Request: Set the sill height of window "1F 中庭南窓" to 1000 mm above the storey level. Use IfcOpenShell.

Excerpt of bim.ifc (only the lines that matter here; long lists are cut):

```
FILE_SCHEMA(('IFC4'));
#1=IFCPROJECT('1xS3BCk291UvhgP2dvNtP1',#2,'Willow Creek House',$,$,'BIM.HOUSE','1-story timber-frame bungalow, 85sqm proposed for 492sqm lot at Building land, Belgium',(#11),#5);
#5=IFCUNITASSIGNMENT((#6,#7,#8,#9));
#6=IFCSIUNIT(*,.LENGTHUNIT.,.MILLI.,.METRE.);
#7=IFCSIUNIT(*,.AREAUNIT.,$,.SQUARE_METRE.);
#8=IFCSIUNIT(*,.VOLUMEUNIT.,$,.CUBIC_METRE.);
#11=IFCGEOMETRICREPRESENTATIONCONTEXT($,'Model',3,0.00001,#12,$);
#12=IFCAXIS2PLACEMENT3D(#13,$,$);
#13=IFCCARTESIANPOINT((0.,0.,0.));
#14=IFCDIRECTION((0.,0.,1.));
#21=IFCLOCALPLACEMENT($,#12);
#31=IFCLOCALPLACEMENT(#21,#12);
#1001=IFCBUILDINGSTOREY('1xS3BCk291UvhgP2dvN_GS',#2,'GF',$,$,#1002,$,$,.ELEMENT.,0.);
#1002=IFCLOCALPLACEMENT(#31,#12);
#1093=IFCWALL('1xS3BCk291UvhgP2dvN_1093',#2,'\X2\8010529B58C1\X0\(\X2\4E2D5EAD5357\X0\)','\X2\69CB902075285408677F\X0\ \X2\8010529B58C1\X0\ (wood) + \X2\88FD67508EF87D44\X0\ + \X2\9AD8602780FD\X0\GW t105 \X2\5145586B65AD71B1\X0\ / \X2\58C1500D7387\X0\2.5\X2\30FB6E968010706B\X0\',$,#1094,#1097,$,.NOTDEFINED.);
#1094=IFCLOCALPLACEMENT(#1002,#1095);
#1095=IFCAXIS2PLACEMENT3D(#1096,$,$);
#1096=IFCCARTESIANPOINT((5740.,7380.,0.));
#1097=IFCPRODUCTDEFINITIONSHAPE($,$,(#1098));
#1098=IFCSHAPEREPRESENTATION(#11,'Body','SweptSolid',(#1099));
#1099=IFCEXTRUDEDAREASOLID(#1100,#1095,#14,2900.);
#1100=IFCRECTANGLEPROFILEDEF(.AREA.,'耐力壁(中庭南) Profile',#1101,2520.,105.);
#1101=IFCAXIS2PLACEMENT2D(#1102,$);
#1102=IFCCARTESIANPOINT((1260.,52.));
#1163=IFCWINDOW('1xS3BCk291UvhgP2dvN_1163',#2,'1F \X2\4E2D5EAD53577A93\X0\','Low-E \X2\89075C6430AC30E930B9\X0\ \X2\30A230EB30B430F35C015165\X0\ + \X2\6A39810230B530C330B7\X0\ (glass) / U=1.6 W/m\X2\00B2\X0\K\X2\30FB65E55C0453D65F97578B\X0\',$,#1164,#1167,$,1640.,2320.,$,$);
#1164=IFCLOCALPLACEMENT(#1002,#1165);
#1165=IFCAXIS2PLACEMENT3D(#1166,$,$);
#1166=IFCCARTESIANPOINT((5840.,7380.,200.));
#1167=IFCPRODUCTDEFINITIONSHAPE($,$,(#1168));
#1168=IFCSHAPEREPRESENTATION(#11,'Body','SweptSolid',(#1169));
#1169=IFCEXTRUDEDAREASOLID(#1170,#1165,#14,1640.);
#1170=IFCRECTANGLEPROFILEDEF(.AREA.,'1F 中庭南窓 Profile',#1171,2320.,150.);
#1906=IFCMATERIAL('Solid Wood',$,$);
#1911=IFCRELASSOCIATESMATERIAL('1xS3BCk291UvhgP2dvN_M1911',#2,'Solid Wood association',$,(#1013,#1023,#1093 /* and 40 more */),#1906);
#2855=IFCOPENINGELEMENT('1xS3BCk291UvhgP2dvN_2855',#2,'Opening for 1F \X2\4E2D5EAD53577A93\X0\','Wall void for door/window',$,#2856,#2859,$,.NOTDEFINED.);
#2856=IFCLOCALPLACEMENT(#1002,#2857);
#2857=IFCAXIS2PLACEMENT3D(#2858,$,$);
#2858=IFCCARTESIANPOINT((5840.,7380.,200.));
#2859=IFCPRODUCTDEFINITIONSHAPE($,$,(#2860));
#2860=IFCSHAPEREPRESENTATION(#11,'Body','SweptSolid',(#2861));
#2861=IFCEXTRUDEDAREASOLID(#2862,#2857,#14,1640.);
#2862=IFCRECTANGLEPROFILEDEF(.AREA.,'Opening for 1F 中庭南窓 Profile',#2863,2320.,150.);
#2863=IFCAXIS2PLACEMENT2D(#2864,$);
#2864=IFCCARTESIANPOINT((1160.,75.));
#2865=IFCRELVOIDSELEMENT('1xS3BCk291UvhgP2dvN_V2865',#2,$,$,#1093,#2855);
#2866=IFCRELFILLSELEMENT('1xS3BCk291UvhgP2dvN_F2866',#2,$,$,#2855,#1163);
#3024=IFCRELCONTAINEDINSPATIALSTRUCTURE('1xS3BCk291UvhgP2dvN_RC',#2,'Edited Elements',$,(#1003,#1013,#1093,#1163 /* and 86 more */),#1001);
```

```python
import numpy as np
import ifcopenshell
import ifcopenshell.api.geometry
import ifcopenshell.geom
import ifcopenshell.util.element
import ifcopenshell.util.placement
import ifcopenshell.util.shape
import ifcopenshell.util.unit

model = ifcopenshell.open("bim.ifc")
unit_scale = ifcopenshell.util.unit.calculate_unit_scale(model)

window = model.by_id(1163)
opening = window.FillsVoids[0].RelatingOpeningElement
storey = ifcopenshell.util.element.get_container(window, ifc_class="IfcBuildingStorey")
level = ifcopenshell.util.placement.get_local_placement(storey.ObjectPlacement)[2, 3]

# The opening's origin need not be at the sill, so measure its lowest point.
shape = ifcopenshell.geom.create_shape(ifcopenshell.geom.settings(), opening)
bottom = ifcopenshell.util.shape.get_shape_bottom_elevation(shape, shape.geometry) / unit_scale
dz = level + 1 / unit_scale - bottom

shift = np.array([0.0, 0.0, dz])
# The window is not placed relative to its opening, so move both.
for product in (opening, window):
    matrix = ifcopenshell.util.placement.get_local_placement(product.ObjectPlacement)
    matrix[:3, 3] += shift
    ifcopenshell.api.geometry.edit_object_placement(model, product=product, matrix=matrix, is_si=False)

print(f"moved by {dz * unit_scale:+.3f} m")

model.write("bim_rev.ifc")
```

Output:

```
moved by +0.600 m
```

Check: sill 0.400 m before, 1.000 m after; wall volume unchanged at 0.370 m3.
